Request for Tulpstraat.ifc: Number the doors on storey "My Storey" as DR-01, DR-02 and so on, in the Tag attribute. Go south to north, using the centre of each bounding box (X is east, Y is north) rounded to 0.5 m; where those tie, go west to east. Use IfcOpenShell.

First a look at what the model holds.

```python
import ifcopenshell
import ifcopenshell.util.element
import ifcopenshell.util.placement

model = ifcopenshell.open("Tulpstraat.ifc")
print(model.schema)
storey = next(s for s in model.by_type("IfcBuildingStorey") if s.Name == "My Storey")
doors = [e for e in ifcopenshell.util.element.get_decomposition(storey) if e.is_a("IfcDoor")]
for e in sorted(doors, key=lambda e: e.id()):
    origin = ifcopenshell.util.placement.get_local_placement(e.ObjectPlacement)[:3, 3]
    print(e.id(), e.Tag, e.Name, origin.round(2) + 0.0, sep=" | ")
```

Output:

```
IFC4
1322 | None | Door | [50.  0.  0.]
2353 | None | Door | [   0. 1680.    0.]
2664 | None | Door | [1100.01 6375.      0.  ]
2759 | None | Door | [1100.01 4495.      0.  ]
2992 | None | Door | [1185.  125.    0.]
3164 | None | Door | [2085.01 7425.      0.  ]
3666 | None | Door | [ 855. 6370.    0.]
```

```python
import ifcopenshell
import ifcopenshell.geom
import ifcopenshell.util.element
import ifcopenshell.util.shape

model = ifcopenshell.open("Tulpstraat.ifc")
settings = ifcopenshell.geom.settings()
settings.set("use-world-coords", True)


def centre(element):
    shape = ifcopenshell.geom.create_shape(settings, element)
    return ifcopenshell.util.shape.get_bbox_centroid(shape.geometry)


storey = next(s for s in model.by_type("IfcBuildingStorey") if s.Name == "My Storey")
doors = [e for e in ifcopenshell.util.element.get_decomposition(storey) if e.is_a("IfcDoor")]

# Insertion points can sit at a corner or the storey origin, so sort by the geometry (in metres).
centres = {e: centre(e) for e in doors}
doors.sort(key=lambda e: (round(centres[e][1] / 0.5), centres[e][0]))

for i, e in enumerate(doors, start=1):
    number = f"DR-{i:02d}"
    e.Tag = number
    print(e.id(), number)

model.write("Tulpstraat_updated.ifc")
```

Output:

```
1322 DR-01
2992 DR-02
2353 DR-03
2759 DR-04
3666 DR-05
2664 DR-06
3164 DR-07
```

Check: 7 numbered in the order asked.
